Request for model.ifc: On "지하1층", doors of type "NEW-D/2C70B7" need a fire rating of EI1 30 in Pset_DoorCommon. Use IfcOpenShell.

First a look at what the model holds.

```python
import ifcopenshell
import ifcopenshell.util.element

model = ifcopenshell.open("model.ifc")
print(model.schema)
storey = next(s for s in model.by_type("IfcBuildingStorey") if s.Name == "지하1층")
doors = [e for e in ifcopenshell.util.element.get_decomposition(storey) if e.is_a("IfcDoor")]
seen = {}
for e in doors:
    element_type = ifcopenshell.util.element.get_type(e)
    key = (element_type.Name if element_type != e and element_type else None, ifcopenshell.util.element.get_pset(e, "Pset_DoorCommon", "FireRating"))
    seen[key] = seen.get(key, 0) + 1
for (name, value), count in sorted(seen.items(), key=str):
    print(count, "x", name, "|", value)
```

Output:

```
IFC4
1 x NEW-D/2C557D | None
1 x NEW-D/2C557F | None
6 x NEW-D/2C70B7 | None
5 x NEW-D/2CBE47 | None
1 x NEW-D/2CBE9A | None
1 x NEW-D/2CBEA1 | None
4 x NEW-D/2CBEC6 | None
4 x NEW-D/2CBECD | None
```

```python
import ifcopenshell
import ifcopenshell.api.pset
import ifcopenshell.util.element

model = ifcopenshell.open("model.ifc")

storey = next(s for s in model.by_type("IfcBuildingStorey") if s.Name == "지하1층")
doors = [e for e in ifcopenshell.util.element.get_decomposition(storey) if e.is_a("IfcDoor")]

count = 0
for e in doors:
    element_type = ifcopenshell.util.element.get_type(e)
    if element_type in (None, e) or element_type.Name != "NEW-D/2C70B7":
        continue
    # add_pset returns the element's existing set when there is one.
    pset = ifcopenshell.api.pset.add_pset(model, product=e, name="Pset_DoorCommon")
    ifcopenshell.api.pset.edit_pset(model, pset=pset, properties={"FireRating": "EI1 30"})
    count += 1

print(count, "doors updated")

model.write("model-out.ifc")
```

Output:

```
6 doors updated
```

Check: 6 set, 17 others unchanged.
